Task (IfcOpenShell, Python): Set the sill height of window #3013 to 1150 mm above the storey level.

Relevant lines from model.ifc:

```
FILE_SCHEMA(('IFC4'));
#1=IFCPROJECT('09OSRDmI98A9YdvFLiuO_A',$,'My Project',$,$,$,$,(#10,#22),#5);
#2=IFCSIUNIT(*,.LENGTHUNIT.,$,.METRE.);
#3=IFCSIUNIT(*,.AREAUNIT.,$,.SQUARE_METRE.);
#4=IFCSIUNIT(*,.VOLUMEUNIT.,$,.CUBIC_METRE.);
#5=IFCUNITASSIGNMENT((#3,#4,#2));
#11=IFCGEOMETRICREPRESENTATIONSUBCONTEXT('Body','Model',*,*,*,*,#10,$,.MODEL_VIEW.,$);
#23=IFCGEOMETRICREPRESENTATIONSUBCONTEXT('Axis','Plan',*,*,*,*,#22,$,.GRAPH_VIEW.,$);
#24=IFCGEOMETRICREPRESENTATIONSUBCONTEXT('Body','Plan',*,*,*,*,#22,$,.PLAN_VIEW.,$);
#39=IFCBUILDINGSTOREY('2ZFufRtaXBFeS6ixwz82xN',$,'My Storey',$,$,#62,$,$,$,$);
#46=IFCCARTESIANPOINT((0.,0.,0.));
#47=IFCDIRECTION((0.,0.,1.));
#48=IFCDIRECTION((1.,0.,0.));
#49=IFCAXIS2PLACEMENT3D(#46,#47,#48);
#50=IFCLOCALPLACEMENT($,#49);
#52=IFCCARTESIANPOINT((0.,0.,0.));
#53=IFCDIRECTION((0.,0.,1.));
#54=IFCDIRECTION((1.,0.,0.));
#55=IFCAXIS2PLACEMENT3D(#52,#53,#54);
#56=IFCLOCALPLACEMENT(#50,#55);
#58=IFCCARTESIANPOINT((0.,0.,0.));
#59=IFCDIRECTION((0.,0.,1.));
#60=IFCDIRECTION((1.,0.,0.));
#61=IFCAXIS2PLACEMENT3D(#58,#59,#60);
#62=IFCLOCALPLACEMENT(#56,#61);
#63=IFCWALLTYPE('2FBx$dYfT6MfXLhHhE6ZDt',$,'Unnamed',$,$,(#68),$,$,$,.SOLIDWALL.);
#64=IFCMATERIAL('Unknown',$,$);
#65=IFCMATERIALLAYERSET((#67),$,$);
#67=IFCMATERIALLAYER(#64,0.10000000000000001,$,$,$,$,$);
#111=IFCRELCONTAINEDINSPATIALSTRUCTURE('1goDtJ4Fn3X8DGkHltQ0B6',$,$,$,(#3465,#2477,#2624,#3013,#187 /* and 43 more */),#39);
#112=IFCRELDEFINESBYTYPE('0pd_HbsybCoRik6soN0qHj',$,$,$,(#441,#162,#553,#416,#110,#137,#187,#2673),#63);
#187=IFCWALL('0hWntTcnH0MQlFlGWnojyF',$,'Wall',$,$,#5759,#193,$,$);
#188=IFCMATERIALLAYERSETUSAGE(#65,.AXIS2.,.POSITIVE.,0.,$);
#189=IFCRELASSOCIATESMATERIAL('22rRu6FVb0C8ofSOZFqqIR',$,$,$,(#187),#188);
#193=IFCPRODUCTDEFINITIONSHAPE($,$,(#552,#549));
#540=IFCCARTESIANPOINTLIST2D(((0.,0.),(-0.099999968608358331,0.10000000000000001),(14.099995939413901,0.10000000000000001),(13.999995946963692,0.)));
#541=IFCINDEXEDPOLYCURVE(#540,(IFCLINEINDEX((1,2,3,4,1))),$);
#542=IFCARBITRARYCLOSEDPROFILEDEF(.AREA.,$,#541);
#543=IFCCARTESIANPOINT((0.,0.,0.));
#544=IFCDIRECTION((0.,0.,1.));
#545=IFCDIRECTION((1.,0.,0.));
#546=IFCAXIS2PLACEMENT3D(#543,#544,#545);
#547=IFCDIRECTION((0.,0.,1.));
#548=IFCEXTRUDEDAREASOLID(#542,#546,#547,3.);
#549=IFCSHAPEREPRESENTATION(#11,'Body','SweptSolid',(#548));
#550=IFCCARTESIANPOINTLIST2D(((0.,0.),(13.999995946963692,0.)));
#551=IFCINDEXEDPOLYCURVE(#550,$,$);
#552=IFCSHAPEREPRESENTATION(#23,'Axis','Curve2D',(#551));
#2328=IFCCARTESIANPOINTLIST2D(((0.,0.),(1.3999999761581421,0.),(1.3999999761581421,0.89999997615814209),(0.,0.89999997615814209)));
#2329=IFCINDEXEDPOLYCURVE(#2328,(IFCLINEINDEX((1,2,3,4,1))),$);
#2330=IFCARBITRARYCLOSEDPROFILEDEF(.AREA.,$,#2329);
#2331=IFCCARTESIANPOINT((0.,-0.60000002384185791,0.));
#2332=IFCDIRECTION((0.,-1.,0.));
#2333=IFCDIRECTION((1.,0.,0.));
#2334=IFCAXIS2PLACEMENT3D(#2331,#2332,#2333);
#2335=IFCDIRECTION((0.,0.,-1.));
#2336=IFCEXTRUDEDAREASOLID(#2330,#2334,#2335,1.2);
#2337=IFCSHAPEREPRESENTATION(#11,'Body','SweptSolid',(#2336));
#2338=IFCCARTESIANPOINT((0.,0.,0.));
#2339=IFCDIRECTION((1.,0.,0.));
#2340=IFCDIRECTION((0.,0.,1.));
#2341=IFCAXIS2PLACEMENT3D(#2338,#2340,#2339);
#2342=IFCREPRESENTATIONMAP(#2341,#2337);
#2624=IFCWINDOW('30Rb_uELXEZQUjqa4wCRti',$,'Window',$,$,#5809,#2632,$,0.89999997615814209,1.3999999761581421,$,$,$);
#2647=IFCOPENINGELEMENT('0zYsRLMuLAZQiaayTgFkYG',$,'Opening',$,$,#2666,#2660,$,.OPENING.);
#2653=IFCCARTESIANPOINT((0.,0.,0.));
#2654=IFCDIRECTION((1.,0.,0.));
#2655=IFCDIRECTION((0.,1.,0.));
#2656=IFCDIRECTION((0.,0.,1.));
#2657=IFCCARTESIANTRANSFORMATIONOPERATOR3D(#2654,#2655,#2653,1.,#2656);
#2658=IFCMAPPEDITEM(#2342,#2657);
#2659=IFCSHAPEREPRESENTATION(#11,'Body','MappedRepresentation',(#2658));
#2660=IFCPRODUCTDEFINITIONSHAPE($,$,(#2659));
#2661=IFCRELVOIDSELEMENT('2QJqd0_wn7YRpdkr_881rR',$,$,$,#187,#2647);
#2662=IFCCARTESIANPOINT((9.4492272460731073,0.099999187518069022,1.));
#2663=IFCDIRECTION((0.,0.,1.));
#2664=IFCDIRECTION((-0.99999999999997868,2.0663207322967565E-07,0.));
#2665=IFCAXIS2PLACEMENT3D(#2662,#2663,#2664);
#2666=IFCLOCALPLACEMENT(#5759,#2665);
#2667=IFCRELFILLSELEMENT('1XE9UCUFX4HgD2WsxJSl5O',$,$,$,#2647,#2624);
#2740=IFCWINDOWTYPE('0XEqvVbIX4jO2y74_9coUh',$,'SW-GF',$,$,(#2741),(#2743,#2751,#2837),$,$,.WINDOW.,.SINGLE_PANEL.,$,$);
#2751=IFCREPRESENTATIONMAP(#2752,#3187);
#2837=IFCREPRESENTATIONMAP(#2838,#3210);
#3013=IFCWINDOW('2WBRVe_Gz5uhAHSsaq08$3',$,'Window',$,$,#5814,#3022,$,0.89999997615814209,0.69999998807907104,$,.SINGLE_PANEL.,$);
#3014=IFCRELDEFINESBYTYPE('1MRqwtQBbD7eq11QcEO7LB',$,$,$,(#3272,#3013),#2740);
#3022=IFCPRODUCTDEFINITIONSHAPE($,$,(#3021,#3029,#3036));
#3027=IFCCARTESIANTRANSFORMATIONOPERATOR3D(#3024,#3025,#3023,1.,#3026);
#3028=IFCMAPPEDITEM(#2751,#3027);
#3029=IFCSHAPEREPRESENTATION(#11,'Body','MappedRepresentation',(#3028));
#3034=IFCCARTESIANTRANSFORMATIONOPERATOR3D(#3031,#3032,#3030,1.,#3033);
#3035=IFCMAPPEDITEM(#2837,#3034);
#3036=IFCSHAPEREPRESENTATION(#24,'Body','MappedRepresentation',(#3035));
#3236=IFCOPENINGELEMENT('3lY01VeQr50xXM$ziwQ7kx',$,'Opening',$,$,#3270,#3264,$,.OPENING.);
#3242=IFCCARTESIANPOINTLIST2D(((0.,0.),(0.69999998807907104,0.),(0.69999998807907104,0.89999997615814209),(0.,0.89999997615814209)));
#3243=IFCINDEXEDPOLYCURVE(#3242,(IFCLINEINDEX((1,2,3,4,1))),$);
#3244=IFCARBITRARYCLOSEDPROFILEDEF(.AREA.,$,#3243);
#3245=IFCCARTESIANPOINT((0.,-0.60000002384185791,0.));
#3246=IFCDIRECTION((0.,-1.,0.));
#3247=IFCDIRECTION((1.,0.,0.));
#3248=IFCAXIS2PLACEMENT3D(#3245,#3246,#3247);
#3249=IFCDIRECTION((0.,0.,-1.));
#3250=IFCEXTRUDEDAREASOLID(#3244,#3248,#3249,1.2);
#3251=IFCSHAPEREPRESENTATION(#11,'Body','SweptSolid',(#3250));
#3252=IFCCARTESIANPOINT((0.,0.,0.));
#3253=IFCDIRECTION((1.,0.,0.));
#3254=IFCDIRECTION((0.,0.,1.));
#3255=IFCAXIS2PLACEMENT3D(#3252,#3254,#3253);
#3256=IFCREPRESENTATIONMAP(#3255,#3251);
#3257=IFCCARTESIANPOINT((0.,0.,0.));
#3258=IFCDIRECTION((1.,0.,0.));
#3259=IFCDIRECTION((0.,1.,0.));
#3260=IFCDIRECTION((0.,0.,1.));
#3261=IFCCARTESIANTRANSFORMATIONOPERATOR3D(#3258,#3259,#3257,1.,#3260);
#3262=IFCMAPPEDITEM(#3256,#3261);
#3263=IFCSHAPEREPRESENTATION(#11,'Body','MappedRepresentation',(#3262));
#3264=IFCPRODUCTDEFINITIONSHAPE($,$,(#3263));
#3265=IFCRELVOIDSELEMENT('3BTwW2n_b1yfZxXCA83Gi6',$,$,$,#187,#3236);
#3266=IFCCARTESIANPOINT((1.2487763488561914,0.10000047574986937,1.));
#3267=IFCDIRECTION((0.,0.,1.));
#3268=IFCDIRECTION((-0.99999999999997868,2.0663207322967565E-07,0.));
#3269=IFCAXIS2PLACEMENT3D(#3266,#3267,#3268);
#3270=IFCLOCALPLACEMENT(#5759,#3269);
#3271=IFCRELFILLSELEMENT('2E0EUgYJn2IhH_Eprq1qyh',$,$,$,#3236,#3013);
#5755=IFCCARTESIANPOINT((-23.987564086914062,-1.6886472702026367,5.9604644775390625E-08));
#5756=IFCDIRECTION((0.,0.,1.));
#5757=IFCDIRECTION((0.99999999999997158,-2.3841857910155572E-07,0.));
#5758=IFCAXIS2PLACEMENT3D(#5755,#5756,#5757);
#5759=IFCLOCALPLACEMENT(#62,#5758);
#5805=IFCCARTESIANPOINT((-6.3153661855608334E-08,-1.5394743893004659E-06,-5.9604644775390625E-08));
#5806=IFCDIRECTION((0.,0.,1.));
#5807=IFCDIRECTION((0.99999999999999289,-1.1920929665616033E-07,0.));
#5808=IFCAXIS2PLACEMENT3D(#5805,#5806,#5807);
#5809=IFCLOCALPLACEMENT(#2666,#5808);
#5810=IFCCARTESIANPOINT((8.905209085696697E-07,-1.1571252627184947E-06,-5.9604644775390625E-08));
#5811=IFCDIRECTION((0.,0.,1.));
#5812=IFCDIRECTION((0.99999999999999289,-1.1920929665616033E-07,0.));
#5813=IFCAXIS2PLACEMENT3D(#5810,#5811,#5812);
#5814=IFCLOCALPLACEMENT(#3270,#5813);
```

```python
import numpy as np
import ifcopenshell
import ifcopenshell.api.geometry
import ifcopenshell.geom
import ifcopenshell.util.element
import ifcopenshell.util.placement
import ifcopenshell.util.shape
import ifcopenshell.util.unit

model = ifcopenshell.open("model.ifc")
unit_scale = ifcopenshell.util.unit.calculate_unit_scale(model)

window = model.by_guid("2WBRVe_Gz5uhAHSsaq08$3")
opening = window.FillsVoids[0].RelatingOpeningElement
storey = ifcopenshell.util.element.get_container(window, ifc_class="IfcBuildingStorey")
level = ifcopenshell.util.placement.get_local_placement(storey.ObjectPlacement)[2, 3]

# The opening's origin need not be at the sill, so measure its lowest point.
shape = ifcopenshell.geom.create_shape(ifcopenshell.geom.settings(), opening)
bottom = ifcopenshell.util.shape.get_shape_bottom_elevation(shape, shape.geometry) / unit_scale
dz = level + 1.15 / unit_scale - bottom

shift = np.array([0.0, 0.0, dz])
# The window is placed relative to its opening, so it follows when the opening moves.
matrix = ifcopenshell.util.placement.get_local_placement(opening.ObjectPlacement)
matrix[:3, 3] += shift
ifcopenshell.api.geometry.edit_object_placement(
    model, product=opening, matrix=matrix, is_si=False, should_transform_children=True
)

print(f"moved by {dz * unit_scale:+.3f} m")

model.write("model_edited.ifc")
```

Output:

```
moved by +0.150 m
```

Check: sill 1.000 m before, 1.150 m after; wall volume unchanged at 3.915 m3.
